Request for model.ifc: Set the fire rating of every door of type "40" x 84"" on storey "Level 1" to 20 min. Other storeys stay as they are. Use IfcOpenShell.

First a look at what the model holds.

```python
import ifcopenshell
import ifcopenshell.util.element

model = ifcopenshell.open("model.ifc")
print(model.schema)
storey = next(s for s in model.by_type("IfcBuildingStorey") if s.Name == "Level 1")
doors = [e for e in ifcopenshell.util.element.get_decomposition(storey) if e.is_a("IfcDoor")]
seen = {}
for e in doors:
    element_type = ifcopenshell.util.element.get_type(e)
    key = (element_type.Name if element_type != e and element_type else None, ifcopenshell.util.element.get_pset(e, "Pset_DoorCommon", "FireRating"))
    seen[key] = seen.get(key, 0) + 1
for (name, value), count in sorted(seen.items(), key=str):
    print(count, "x", name, "|", value)
```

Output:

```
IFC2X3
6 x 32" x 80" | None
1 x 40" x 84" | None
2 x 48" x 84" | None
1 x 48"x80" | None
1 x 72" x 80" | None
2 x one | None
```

```python
import ifcopenshell
import ifcopenshell.api.pset
import ifcopenshell.util.element

model = ifcopenshell.open("model.ifc")

storey = next(s for s in model.by_type("IfcBuildingStorey") if s.Name == "Level 1")
doors = [e for e in ifcopenshell.util.element.get_decomposition(storey) if e.is_a("IfcDoor")]

count = 0
for e in doors:
    element_type = ifcopenshell.util.element.get_type(e)
    if element_type in (None, e) or element_type.Name != '40" x 84"':
        continue
    # add_pset returns the element's existing set when there is one.
    pset = ifcopenshell.api.pset.add_pset(model, product=e, name="Pset_DoorCommon")
    ifcopenshell.api.pset.edit_pset(model, pset=pset, properties={"FireRating": "20 min"})
    count += 1

print(count, "doors updated")

model.write("model_rev.ifc")
```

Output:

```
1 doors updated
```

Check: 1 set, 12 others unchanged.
